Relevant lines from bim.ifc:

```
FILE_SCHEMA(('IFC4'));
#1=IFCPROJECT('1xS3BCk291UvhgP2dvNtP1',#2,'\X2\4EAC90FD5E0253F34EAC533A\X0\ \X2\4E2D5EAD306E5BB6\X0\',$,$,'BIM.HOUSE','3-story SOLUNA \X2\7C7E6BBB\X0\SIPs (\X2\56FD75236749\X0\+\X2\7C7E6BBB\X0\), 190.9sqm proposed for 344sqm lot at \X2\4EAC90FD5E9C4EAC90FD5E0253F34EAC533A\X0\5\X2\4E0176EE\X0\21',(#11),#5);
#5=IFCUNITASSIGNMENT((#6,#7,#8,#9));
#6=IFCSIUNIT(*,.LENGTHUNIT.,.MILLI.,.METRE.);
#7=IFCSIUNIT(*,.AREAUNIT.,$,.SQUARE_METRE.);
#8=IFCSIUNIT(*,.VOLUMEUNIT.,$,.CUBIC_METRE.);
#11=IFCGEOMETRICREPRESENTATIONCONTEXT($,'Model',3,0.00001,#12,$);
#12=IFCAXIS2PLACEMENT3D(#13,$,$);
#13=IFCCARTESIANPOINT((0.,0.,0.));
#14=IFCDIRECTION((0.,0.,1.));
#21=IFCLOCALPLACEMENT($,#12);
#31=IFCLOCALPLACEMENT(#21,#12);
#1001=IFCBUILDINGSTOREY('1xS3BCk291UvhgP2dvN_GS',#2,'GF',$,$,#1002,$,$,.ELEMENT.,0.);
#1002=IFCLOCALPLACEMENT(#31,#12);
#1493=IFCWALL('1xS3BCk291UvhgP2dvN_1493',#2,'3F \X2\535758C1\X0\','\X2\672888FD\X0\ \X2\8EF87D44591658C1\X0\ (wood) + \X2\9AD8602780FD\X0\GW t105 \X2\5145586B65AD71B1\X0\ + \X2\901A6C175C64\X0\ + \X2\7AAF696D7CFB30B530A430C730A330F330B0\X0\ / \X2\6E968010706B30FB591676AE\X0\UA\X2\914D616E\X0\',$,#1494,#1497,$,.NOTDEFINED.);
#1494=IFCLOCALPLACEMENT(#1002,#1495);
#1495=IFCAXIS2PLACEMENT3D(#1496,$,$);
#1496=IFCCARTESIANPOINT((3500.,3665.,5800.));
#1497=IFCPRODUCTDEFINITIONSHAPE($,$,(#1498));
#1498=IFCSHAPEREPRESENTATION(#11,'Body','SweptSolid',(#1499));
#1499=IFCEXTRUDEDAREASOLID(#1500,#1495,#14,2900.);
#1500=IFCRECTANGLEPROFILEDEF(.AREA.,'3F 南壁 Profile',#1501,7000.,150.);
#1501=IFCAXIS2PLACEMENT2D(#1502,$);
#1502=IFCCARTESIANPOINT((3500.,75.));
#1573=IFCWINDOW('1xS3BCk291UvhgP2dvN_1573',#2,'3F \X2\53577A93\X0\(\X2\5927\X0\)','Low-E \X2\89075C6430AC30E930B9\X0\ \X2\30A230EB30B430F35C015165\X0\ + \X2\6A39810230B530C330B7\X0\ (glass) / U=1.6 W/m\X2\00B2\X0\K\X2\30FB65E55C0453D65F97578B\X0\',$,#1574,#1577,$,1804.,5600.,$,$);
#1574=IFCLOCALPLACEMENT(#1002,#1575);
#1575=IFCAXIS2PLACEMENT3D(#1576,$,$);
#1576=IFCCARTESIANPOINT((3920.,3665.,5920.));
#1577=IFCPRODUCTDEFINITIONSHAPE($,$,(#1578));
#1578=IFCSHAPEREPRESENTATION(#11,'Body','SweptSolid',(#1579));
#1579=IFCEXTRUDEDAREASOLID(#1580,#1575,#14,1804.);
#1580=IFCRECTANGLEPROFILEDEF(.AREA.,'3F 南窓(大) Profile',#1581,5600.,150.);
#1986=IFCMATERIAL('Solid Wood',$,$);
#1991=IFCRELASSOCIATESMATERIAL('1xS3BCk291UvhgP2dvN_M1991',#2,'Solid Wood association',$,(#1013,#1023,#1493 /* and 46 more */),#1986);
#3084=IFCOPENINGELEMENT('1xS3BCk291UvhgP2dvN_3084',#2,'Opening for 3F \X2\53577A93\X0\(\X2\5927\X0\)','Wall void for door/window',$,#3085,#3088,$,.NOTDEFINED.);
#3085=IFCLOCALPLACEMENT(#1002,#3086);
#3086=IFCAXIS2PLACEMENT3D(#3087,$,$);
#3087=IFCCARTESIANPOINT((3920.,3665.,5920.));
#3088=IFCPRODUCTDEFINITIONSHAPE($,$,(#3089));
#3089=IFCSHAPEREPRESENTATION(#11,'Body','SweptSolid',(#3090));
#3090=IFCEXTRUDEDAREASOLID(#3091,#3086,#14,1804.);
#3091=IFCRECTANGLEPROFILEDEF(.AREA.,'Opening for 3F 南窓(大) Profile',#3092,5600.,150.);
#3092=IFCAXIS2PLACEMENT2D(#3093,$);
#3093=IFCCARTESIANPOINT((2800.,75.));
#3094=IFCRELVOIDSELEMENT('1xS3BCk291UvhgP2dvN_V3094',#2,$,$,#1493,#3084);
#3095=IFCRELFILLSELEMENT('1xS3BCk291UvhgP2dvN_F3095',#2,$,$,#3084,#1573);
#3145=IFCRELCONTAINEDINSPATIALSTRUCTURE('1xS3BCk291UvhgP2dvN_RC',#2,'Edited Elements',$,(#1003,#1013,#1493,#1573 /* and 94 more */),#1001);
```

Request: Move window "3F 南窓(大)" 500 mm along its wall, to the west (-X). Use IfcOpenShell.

```python
import ifcopenshell
import ifcopenshell.api.geometry
import ifcopenshell.util.placement

model = ifcopenshell.open("bim.ifc")

window = model.by_guid("1xS3BCk291UvhgP2dvN_1573")
opening = window.FillsVoids[0].RelatingOpeningElement
wall = opening.VoidsElements[0].RelatingBuildingElement

wall_matrix = ifcopenshell.util.placement.get_local_placement(wall.ObjectPlacement)
shift = wall_matrix[:3, 0] * -500.0
before = ifcopenshell.util.placement.get_local_placement(window.ObjectPlacement)[:3, 3].copy()

# The window is not placed relative to its opening, so move both.
for product in (opening, window):
    matrix = ifcopenshell.util.placement.get_local_placement(product.ObjectPlacement)
    matrix[:3, 3] += shift
    ifcopenshell.api.geometry.edit_object_placement(model, product=product, matrix=matrix, is_si=False)

after = ifcopenshell.util.placement.get_local_placement(window.ObjectPlacement)[:3, 3]
print("window moved by", (after - before).round(3) + 0.0)

model.write("bim_rev.ifc")
```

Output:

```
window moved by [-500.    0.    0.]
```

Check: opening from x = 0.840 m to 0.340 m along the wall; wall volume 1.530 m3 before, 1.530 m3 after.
